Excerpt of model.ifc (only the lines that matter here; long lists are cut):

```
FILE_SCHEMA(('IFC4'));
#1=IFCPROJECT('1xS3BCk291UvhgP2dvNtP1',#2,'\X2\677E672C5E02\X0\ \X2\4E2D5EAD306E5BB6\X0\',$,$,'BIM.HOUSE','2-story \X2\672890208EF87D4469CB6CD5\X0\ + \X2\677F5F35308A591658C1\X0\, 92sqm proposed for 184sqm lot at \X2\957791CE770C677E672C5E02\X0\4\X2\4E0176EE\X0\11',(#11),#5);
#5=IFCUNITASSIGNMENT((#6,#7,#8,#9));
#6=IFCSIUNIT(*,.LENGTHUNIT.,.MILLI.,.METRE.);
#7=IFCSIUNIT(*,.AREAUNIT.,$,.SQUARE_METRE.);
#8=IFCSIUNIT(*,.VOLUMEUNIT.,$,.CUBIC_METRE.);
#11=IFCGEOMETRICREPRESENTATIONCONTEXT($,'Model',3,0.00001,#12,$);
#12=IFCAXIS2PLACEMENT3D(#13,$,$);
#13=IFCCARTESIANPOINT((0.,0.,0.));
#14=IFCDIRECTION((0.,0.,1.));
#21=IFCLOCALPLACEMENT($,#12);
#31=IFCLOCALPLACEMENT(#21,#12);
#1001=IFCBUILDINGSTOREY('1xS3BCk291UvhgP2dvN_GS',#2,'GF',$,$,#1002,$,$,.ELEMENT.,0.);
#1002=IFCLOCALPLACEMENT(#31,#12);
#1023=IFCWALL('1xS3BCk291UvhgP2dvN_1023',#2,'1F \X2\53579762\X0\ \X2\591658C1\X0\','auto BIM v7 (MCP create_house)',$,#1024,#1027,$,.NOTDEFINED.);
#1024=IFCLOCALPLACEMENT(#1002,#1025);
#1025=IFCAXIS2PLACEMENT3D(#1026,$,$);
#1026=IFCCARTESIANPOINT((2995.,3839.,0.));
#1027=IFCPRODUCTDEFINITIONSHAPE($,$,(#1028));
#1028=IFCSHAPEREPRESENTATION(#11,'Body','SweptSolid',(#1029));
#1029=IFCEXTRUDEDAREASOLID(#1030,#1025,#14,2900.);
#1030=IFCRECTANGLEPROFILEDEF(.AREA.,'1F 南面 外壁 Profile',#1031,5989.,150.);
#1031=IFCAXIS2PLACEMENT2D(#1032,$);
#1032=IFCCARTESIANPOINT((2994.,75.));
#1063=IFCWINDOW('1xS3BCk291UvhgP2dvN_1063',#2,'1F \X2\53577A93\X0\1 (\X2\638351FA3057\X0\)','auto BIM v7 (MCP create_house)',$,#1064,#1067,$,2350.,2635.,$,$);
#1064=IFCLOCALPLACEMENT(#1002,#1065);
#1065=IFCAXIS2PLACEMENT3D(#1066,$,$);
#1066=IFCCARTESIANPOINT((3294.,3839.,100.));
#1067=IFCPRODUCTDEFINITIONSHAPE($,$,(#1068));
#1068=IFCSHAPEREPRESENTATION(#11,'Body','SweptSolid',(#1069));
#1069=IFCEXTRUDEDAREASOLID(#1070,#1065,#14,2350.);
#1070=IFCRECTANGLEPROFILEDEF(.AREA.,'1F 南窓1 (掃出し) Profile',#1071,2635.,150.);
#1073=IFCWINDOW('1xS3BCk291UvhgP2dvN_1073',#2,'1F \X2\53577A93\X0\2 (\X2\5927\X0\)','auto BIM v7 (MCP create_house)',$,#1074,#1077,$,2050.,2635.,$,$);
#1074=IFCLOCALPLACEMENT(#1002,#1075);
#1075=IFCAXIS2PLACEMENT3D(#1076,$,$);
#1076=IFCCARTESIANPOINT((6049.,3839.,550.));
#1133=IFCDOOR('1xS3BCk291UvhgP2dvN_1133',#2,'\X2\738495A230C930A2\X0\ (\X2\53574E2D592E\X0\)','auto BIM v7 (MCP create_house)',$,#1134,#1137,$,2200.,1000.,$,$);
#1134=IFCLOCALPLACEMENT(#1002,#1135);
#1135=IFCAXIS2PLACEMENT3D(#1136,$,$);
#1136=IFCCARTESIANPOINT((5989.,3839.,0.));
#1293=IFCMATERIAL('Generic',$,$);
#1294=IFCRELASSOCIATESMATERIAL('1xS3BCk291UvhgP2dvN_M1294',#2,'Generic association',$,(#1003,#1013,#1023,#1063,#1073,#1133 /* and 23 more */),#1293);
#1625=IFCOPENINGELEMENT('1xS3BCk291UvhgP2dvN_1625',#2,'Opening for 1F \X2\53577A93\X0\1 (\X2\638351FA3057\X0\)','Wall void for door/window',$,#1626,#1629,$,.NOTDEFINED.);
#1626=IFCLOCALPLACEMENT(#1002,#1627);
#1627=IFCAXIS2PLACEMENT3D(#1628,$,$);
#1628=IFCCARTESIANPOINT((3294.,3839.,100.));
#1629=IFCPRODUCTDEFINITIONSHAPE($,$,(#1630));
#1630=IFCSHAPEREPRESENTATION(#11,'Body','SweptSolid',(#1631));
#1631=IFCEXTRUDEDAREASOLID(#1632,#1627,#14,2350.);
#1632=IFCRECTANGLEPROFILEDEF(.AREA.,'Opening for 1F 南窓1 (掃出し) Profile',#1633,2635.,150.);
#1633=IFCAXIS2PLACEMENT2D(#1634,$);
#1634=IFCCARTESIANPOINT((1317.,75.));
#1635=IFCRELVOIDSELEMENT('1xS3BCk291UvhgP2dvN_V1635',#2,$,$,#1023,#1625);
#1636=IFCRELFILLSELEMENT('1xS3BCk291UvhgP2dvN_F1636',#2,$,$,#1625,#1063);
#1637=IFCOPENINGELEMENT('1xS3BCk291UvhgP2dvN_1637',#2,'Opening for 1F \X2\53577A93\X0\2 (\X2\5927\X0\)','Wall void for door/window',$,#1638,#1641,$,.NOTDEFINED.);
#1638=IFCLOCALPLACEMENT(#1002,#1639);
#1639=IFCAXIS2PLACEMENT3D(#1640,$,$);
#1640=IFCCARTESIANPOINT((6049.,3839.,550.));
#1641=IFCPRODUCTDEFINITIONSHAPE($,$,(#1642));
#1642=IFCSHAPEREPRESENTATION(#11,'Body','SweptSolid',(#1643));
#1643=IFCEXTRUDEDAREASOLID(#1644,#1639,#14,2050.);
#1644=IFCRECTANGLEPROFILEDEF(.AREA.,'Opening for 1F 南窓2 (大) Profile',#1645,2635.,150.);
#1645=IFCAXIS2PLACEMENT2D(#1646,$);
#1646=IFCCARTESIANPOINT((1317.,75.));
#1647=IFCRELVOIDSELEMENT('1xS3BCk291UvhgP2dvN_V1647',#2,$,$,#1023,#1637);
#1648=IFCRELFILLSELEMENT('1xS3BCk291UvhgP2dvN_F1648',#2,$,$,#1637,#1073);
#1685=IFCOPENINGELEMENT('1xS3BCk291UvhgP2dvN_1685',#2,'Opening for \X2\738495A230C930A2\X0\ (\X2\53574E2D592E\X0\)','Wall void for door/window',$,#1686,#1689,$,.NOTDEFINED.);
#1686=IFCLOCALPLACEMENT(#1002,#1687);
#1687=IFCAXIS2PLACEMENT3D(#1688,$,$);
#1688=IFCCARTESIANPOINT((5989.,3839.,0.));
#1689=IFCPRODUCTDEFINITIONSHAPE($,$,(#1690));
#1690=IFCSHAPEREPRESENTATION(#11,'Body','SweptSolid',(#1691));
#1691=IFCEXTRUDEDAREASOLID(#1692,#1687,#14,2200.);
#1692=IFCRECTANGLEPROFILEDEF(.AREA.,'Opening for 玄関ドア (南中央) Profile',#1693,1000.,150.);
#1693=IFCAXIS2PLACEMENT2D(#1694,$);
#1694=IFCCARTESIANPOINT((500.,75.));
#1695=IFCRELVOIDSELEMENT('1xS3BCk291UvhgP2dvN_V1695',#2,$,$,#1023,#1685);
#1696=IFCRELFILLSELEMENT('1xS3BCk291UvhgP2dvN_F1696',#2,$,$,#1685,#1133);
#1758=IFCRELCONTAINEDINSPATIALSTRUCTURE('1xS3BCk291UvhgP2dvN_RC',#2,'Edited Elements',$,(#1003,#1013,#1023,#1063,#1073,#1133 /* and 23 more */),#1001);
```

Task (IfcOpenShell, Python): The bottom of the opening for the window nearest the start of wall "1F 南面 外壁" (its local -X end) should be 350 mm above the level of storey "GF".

```python
import numpy as np
import ifcopenshell
import ifcopenshell.api.geometry
import ifcopenshell.geom
import ifcopenshell.util.element
import ifcopenshell.util.placement
import ifcopenshell.util.shape
import ifcopenshell.util.unit

model = ifcopenshell.open("model.ifc")
unit_scale = ifcopenshell.util.unit.calculate_unit_scale(model)

window = model.by_guid("1xS3BCk291UvhgP2dvN_1063")
opening = window.FillsVoids[0].RelatingOpeningElement
storey = ifcopenshell.util.element.get_container(window, ifc_class="IfcBuildingStorey")
level = ifcopenshell.util.placement.get_local_placement(storey.ObjectPlacement)[2, 3]

# The opening's origin need not be at the sill, so measure its lowest point.
shape = ifcopenshell.geom.create_shape(ifcopenshell.geom.settings(), opening)
bottom = ifcopenshell.util.shape.get_shape_bottom_elevation(shape, shape.geometry) / unit_scale
dz = level + 0.35 / unit_scale - bottom

shift = np.array([0.0, 0.0, dz])
# The window is not placed relative to its opening, so move both.
for product in (opening, window):
    matrix = ifcopenshell.util.placement.get_local_placement(product.ObjectPlacement)
    matrix[:3, 3] += shift
    ifcopenshell.api.geometry.edit_object_placement(model, product=product, matrix=matrix, is_si=False)

print(f"moved by {dz * unit_scale:+.3f} m")

model.write("model_rev.ifc")
```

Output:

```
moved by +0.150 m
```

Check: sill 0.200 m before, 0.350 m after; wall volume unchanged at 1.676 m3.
